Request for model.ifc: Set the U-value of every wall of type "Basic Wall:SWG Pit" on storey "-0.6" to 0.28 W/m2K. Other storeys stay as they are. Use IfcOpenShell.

First a look at what the model holds.

```python
import ifcopenshell
import ifcopenshell.util.element

model = ifcopenshell.open("model.ifc")
print(model.schema)
storey = next(s for s in model.by_type("IfcBuildingStorey") if s.Name == "-0.6")
walls = [e for e in ifcopenshell.util.element.get_decomposition(storey) if e.is_a("IfcWall")]
seen = {}
for e in walls:
    element_type = ifcopenshell.util.element.get_type(e)
    key = (element_type.Name if element_type != e and element_type else None, ifcopenshell.util.element.get_pset(e, "Pset_WallCommon", "ThermalTransmittance"))
    seen[key] = seen.get(key, 0) + 1
for (name, value), count in sorted(seen.items(), key=str):
    print(count, "x", name, "|", value)
```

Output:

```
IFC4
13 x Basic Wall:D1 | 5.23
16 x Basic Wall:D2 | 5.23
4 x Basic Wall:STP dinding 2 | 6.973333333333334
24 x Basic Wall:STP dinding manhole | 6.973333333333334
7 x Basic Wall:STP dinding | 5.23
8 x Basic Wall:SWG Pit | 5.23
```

```python
import ifcopenshell
import ifcopenshell.api.pset
import ifcopenshell.util.element

model = ifcopenshell.open("model.ifc")

storey = next(s for s in model.by_type("IfcBuildingStorey") if s.Name == "-0.6")
walls = [e for e in ifcopenshell.util.element.get_decomposition(storey) if e.is_a("IfcWall")]

count = 0
for e in walls:
    element_type = ifcopenshell.util.element.get_type(e)
    if element_type in (None, e) or element_type.Name != "Basic Wall:SWG Pit":
        continue
    # add_pset returns the element's existing set when there is one.
    pset = ifcopenshell.api.pset.add_pset(model, product=e, name="Pset_WallCommon")
    ifcopenshell.api.pset.edit_pset(model, pset=pset, properties={"ThermalTransmittance": 0.28})
    count += 1

print(count, "walls updated")

model.write("model_edited.ifc")
```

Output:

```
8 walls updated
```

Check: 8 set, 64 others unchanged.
